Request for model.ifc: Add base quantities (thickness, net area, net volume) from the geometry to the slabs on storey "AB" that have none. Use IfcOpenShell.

First a look at what the model holds.

```python
import ifcopenshell
import ifcopenshell.util.element
import ifcopenshell.util.unit

model = ifcopenshell.open("model.ifc")
print(model.schema)
for unit_type in ("LENGTHUNIT", "AREAUNIT", "VOLUMEUNIT"):
    print(unit_type, ifcopenshell.util.unit.calculate_unit_scale(model, unit_type))
storey = next(s for s in model.by_type("IfcBuildingStorey") if s.Name == "AB")
slabs = [e for e in ifcopenshell.util.element.get_decomposition(storey) if e.is_a("IfcSlab")]
for e in sorted(slabs, key=lambda e: e.id()):
    print(e.id(), e.is_a(), e.Name, list(ifcopenshell.util.element.get_psets(e, qtos_only=True)), sep=" | ")
```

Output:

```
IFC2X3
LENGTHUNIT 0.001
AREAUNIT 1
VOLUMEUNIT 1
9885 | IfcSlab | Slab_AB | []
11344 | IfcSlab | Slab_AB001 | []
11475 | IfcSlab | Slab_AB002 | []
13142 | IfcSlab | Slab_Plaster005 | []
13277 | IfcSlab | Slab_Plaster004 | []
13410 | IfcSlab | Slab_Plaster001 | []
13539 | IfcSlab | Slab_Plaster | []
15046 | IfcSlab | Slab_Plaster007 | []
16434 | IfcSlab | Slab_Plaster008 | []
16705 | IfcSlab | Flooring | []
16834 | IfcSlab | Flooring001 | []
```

```python
import ifcopenshell
import ifcopenshell.api.pset
import ifcopenshell.geom
import ifcopenshell.util.element
import ifcopenshell.util.shape
import ifcopenshell.util.unit

model = ifcopenshell.open("model.ifc")
unit_scale = ifcopenshell.util.unit.calculate_unit_scale(model)
area_scale = ifcopenshell.util.unit.calculate_unit_scale(model, "AREAUNIT")
volume_scale = ifcopenshell.util.unit.calculate_unit_scale(model, "VOLUMEUNIT")
settings = ifcopenshell.geom.settings()

storey = next(s for s in model.by_type("IfcBuildingStorey") if s.Name == "AB")
slabs = [e for e in ifcopenshell.util.element.get_decomposition(storey) if e.is_a("IfcSlab")]

for e in sorted(slabs, key=lambda e: e.id()):
    if ifcopenshell.util.element.get_psets(e, qtos_only=True, should_inherit=False):
        continue
    # Geometry comes back in metres, in the element's own axes.
    shape = ifcopenshell.geom.create_shape(settings, e)
    values = {
        "Width": ifcopenshell.util.shape.get_z(shape.geometry) / unit_scale,
        "NetArea": ifcopenshell.util.shape.get_footprint_area(shape.geometry) / area_scale,
        "NetVolume": ifcopenshell.util.shape.get_volume(shape.geometry) / volume_scale,
    }
    qto = ifcopenshell.api.pset.add_qto(model, product=e, name="BaseQuantities")
    ifcopenshell.api.pset.edit_qto(model, qto=qto, properties=values)
    print(e.id(), {k: round(v, 3) for k, v in values.items()})

model.write("model_rev.ifc")
```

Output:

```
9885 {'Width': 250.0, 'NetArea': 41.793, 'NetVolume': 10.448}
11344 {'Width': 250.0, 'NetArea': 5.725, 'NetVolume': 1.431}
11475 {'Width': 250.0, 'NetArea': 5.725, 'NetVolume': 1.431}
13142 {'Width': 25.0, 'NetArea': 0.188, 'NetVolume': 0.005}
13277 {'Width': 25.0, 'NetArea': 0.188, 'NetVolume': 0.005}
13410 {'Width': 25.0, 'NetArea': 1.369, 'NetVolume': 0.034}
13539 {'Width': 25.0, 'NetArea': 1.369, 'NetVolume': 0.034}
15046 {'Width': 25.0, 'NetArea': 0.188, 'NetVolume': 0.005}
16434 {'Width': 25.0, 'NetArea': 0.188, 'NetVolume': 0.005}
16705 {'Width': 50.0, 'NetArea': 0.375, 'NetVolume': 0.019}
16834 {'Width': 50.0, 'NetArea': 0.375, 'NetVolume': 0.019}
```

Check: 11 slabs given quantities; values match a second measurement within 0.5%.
